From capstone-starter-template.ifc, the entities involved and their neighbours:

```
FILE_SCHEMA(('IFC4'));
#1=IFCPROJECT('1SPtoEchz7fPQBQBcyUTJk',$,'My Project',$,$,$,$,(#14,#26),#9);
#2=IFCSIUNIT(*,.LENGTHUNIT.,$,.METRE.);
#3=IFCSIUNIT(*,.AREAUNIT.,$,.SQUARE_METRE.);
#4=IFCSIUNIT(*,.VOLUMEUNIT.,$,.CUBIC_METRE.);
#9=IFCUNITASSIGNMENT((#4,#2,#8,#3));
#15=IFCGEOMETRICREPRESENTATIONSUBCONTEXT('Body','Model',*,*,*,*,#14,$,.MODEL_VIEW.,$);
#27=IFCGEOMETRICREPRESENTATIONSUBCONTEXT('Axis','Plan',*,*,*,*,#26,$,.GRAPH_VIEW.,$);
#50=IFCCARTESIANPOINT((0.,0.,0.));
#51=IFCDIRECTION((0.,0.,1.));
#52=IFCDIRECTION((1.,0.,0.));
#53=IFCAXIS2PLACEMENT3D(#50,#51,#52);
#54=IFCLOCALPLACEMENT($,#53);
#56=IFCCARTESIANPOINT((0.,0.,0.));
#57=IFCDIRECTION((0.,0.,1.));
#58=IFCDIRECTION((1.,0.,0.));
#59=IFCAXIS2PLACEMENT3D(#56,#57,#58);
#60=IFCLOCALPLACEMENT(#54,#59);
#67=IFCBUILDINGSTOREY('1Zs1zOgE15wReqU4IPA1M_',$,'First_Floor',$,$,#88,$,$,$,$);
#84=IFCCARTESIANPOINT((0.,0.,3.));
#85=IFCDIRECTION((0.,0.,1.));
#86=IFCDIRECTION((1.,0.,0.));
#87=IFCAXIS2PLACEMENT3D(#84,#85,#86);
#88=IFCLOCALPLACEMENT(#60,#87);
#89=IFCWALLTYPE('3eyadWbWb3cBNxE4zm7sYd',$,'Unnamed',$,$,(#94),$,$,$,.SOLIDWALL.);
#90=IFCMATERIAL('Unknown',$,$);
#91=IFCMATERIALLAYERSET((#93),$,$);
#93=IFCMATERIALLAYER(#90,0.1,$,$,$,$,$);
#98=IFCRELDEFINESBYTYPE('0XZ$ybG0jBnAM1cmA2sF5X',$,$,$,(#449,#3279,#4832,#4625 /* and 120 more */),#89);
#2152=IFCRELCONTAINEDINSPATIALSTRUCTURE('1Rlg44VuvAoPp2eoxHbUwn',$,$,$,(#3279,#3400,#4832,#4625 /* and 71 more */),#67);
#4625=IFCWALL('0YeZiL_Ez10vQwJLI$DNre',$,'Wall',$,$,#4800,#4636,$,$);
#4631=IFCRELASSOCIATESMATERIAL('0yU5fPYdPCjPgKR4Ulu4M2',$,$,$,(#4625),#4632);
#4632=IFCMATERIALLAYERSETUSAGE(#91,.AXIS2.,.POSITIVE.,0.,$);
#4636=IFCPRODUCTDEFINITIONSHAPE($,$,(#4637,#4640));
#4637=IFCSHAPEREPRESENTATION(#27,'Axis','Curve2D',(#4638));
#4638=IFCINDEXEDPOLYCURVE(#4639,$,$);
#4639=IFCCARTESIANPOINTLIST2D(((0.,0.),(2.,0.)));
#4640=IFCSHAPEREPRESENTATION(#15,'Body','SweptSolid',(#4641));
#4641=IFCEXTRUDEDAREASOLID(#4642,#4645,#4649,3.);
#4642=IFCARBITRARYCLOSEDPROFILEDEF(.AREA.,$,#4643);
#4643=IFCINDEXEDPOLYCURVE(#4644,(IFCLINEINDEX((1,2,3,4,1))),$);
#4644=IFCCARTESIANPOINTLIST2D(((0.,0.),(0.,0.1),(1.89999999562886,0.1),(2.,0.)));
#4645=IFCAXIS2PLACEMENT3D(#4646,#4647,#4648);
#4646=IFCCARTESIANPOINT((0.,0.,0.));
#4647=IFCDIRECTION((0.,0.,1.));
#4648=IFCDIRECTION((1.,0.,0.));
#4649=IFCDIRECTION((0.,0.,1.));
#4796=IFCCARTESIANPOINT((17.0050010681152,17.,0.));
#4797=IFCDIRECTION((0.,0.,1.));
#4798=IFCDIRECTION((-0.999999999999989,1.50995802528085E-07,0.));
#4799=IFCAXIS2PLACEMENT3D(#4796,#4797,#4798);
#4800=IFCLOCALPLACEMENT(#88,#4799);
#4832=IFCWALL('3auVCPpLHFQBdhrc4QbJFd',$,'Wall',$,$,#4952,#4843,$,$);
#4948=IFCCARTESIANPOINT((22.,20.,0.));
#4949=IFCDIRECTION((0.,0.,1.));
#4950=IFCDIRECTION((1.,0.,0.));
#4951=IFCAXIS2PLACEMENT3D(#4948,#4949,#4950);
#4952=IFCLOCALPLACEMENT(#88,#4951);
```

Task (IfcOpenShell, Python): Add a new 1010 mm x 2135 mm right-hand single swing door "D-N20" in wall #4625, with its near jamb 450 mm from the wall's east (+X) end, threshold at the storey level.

```python
import numpy as np
import ifcopenshell
import ifcopenshell.api.feature
import ifcopenshell.api.geometry
import ifcopenshell.api.root
import ifcopenshell.api.spatial
import ifcopenshell.geom
import ifcopenshell.util.element
import ifcopenshell.util.placement
import ifcopenshell.util.representation
import ifcopenshell.util.shape
import ifcopenshell.util.unit

model = ifcopenshell.open("capstone-starter-template.ifc")
unit_scale = ifcopenshell.util.unit.calculate_unit_scale(model)
settings = ifcopenshell.geom.settings()


def volume(element):
    """Net volume in cubic metres, openings subtracted."""
    shape = ifcopenshell.geom.create_shape(settings, element)
    return ifcopenshell.util.shape.get_volume(shape.geometry)


wall = model.by_guid("0YeZiL_Ez10vQwJLI$DNre")
storey = ifcopenshell.util.element.get_container(wall, ifc_class="IfcBuildingStorey")
context = ifcopenshell.util.representation.get_context(model, "Model", "Body", "MODEL_VIEW")
before = volume(wall)

width, height, from_end, sill = 1.01, 2.135, 0.45, 0.0  # metres

# The wall runs along its own X axis, and the end named is its -X end.
wall_shape = ifcopenshell.geom.create_shape(settings, wall)
x, y, z = ifcopenshell.util.shape.get_vertices(wall_shape.geometry).T
start = x.min() + from_end
face, thickness = float(y.min()), float(y.max() - y.min())
wall_matrix = ifcopenshell.util.placement.get_local_placement(wall.ObjectPlacement)
level = ifcopenshell.util.placement.get_local_placement(storey.ObjectPlacement)[2, 3]


def in_wall(x, y):
    """Placement at x, y metres in the wall's axes, at sill height."""
    matrix = wall_matrix.copy()
    matrix[:, 3] = wall_matrix @ np.array([x / unit_scale, y / unit_scale, 0.0, 1.0])
    matrix[2, 3] = level + sill / unit_scale
    return matrix


# Opening: a box that overshoots both wall faces by 50 mm.
opening = ifcopenshell.api.root.create_entity(model, ifc_class="IfcOpeningElement", predefined_type="OPENING")
box = ifcopenshell.api.geometry.add_wall_representation(
    model, context=context, length=width, height=height, thickness=thickness + 0.1
)
ifcopenshell.api.geometry.assign_representation(model, product=opening, representation=box)
ifcopenshell.api.geometry.edit_object_placement(model, product=opening, matrix=in_wall(start, face - 0.05), is_si=False)
ifcopenshell.api.feature.add_feature(model, feature=opening, element=wall)

door = ifcopenshell.api.root.create_entity(model, ifc_class="IfcDoor", name="D-N20", predefined_type="DOOR")
door.OverallWidth, door.OverallHeight = width / unit_scale, height / unit_scale
door.OperationType = "SINGLE_SWING_RIGHT"
body = ifcopenshell.api.geometry.add_door_representation(
    model,
    context=context,
    overall_width=door.OverallWidth,
    overall_height=door.OverallHeight,
    operation_type="SINGLE_SWING_RIGHT",
    lining_properties={"LiningDepth": thickness / unit_scale, "ThresholdDepth": thickness / unit_scale},
)
ifcopenshell.api.geometry.assign_representation(model, product=door, representation=body)
ifcopenshell.api.spatial.assign_container(model, products=[door], relating_structure=storey)
ifcopenshell.api.feature.add_filling(model, opening=opening, element=door)

# The lining spans the wall, so the door starts at the wall face.
ifcopenshell.api.geometry.edit_object_placement(model, product=door, matrix=in_wall(start, face), is_si=False)

after = volume(wall)

print(f"wall volume {before:.3f} -> {after:.3f} m3")

model.write("capstone-starter-template-out.ifc")
```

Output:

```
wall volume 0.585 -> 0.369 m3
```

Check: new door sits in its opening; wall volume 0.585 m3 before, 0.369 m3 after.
